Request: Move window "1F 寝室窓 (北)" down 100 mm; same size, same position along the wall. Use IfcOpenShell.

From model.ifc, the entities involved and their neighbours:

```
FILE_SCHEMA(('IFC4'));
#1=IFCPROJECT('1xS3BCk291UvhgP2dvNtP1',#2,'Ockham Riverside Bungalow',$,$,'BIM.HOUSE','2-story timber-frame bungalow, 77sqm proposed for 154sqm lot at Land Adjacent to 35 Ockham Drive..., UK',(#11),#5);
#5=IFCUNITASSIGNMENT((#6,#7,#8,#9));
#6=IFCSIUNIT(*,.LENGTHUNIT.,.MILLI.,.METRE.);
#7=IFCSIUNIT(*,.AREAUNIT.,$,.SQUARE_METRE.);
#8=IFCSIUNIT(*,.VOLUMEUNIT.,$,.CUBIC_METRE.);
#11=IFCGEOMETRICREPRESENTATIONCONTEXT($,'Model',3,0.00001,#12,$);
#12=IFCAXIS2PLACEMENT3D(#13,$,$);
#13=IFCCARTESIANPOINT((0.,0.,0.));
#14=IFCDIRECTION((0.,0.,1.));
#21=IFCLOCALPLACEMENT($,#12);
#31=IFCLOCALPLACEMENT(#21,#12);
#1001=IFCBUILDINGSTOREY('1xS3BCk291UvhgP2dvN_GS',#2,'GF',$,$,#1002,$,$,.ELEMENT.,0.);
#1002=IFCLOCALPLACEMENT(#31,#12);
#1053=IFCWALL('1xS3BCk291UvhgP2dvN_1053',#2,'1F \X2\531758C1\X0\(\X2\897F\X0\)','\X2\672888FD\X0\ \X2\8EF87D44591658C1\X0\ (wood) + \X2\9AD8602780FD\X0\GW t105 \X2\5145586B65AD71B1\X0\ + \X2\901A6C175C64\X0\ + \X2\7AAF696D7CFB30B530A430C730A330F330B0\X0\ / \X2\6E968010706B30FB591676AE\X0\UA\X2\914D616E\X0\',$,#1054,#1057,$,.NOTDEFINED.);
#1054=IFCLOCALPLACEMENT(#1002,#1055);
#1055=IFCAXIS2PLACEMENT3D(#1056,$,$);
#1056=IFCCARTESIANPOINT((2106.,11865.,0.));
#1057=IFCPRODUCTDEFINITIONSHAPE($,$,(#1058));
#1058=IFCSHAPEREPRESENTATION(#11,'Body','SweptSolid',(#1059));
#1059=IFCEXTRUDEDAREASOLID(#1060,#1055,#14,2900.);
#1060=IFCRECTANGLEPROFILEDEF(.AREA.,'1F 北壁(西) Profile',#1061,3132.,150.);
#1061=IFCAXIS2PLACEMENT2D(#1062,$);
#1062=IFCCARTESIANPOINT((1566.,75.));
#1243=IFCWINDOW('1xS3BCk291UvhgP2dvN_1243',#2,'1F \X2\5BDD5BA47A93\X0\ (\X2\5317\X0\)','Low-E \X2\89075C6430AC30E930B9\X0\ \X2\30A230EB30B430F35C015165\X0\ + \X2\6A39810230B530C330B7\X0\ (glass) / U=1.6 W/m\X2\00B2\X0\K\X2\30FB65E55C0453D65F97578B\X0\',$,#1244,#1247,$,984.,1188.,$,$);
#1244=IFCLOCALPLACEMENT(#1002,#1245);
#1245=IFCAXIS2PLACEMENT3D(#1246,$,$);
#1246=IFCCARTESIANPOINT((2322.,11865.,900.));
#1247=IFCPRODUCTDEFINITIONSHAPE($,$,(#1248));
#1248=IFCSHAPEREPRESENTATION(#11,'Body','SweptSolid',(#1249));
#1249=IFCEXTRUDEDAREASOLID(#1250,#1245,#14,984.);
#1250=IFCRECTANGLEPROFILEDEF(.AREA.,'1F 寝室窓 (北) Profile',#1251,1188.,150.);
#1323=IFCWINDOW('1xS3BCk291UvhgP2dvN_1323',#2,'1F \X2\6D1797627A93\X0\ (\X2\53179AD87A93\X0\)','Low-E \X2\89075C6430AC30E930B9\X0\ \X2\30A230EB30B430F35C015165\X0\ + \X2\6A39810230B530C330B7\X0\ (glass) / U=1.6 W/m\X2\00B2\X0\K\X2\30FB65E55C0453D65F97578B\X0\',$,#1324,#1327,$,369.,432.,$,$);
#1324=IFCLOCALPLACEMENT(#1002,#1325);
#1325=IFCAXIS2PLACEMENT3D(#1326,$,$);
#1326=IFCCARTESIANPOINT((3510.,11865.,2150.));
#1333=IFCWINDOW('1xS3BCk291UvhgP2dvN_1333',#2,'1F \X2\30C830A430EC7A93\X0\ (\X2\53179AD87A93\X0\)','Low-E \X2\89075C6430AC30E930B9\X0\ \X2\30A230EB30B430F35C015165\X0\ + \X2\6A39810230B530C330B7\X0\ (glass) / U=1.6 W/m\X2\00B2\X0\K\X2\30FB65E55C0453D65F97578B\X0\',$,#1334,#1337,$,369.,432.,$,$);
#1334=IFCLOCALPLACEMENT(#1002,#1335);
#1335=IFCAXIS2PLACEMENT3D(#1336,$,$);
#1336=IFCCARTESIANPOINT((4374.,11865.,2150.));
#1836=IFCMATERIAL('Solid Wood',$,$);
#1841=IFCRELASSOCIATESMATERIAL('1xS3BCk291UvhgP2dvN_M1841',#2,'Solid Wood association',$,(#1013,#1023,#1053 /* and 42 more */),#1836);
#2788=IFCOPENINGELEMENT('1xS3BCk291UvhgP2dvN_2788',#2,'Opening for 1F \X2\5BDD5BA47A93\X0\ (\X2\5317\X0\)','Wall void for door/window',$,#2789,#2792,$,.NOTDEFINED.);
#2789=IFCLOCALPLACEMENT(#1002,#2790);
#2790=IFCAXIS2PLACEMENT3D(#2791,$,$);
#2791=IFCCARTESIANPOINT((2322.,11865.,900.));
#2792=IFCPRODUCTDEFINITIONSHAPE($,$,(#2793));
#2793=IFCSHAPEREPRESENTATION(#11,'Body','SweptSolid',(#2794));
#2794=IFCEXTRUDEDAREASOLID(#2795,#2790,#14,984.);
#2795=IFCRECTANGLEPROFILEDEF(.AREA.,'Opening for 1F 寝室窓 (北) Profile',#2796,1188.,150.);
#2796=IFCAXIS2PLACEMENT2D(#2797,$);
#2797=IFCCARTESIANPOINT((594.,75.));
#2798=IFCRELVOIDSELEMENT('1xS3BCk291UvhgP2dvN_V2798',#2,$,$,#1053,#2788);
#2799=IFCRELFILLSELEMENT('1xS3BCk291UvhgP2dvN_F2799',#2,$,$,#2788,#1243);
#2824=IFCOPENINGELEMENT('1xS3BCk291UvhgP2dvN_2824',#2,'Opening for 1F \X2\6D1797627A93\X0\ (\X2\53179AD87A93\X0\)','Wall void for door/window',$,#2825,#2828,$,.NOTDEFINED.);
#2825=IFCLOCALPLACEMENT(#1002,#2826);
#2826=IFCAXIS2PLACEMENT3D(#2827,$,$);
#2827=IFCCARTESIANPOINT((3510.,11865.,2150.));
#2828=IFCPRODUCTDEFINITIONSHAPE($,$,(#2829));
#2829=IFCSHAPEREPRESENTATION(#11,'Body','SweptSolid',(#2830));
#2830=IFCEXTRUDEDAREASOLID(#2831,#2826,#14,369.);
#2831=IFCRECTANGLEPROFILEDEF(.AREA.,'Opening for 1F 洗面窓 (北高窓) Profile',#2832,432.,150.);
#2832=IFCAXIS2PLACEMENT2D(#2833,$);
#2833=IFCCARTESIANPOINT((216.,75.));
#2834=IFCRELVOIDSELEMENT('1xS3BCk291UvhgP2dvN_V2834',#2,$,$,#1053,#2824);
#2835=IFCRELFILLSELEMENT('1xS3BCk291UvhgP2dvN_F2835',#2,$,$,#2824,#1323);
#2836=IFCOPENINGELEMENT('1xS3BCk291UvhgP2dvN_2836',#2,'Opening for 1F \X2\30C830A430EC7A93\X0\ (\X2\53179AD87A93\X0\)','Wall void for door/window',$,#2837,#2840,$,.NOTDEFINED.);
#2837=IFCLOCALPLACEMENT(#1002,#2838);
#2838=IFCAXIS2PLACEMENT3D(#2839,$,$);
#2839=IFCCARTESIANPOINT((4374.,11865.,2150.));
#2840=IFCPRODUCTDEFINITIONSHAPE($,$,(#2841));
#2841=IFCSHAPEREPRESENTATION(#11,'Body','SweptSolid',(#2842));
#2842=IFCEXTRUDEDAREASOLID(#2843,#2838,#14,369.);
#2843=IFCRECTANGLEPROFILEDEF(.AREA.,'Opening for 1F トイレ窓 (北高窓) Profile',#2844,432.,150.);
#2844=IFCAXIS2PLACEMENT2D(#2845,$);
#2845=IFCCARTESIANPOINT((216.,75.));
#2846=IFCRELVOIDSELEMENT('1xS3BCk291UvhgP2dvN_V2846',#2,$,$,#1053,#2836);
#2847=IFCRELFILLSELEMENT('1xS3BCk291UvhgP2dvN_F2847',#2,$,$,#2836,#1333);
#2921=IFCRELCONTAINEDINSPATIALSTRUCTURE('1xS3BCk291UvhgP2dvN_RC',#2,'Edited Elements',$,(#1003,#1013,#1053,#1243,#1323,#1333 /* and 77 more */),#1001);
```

```python
import numpy as np
import ifcopenshell
import ifcopenshell.api.geometry
import ifcopenshell.util.placement
import ifcopenshell.util.unit

model = ifcopenshell.open("model.ifc")
unit_scale = ifcopenshell.util.unit.calculate_unit_scale(model)

window = model.by_guid("1xS3BCk291UvhgP2dvN_1243")
opening = window.FillsVoids[0].RelatingOpeningElement
dz = -0.1 / unit_scale

shift = np.array([0.0, 0.0, dz])
# The window is not placed relative to its opening, so move both.
for product in (opening, window):
    matrix = ifcopenshell.util.placement.get_local_placement(product.ObjectPlacement)
    matrix[:3, 3] += shift
    ifcopenshell.api.geometry.edit_object_placement(model, product=product, matrix=matrix, is_si=False)

print(f"moved by {dz * unit_scale:+.3f} m")

model.write("model_edited.ifc")
```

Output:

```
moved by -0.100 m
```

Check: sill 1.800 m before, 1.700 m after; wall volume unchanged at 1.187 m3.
